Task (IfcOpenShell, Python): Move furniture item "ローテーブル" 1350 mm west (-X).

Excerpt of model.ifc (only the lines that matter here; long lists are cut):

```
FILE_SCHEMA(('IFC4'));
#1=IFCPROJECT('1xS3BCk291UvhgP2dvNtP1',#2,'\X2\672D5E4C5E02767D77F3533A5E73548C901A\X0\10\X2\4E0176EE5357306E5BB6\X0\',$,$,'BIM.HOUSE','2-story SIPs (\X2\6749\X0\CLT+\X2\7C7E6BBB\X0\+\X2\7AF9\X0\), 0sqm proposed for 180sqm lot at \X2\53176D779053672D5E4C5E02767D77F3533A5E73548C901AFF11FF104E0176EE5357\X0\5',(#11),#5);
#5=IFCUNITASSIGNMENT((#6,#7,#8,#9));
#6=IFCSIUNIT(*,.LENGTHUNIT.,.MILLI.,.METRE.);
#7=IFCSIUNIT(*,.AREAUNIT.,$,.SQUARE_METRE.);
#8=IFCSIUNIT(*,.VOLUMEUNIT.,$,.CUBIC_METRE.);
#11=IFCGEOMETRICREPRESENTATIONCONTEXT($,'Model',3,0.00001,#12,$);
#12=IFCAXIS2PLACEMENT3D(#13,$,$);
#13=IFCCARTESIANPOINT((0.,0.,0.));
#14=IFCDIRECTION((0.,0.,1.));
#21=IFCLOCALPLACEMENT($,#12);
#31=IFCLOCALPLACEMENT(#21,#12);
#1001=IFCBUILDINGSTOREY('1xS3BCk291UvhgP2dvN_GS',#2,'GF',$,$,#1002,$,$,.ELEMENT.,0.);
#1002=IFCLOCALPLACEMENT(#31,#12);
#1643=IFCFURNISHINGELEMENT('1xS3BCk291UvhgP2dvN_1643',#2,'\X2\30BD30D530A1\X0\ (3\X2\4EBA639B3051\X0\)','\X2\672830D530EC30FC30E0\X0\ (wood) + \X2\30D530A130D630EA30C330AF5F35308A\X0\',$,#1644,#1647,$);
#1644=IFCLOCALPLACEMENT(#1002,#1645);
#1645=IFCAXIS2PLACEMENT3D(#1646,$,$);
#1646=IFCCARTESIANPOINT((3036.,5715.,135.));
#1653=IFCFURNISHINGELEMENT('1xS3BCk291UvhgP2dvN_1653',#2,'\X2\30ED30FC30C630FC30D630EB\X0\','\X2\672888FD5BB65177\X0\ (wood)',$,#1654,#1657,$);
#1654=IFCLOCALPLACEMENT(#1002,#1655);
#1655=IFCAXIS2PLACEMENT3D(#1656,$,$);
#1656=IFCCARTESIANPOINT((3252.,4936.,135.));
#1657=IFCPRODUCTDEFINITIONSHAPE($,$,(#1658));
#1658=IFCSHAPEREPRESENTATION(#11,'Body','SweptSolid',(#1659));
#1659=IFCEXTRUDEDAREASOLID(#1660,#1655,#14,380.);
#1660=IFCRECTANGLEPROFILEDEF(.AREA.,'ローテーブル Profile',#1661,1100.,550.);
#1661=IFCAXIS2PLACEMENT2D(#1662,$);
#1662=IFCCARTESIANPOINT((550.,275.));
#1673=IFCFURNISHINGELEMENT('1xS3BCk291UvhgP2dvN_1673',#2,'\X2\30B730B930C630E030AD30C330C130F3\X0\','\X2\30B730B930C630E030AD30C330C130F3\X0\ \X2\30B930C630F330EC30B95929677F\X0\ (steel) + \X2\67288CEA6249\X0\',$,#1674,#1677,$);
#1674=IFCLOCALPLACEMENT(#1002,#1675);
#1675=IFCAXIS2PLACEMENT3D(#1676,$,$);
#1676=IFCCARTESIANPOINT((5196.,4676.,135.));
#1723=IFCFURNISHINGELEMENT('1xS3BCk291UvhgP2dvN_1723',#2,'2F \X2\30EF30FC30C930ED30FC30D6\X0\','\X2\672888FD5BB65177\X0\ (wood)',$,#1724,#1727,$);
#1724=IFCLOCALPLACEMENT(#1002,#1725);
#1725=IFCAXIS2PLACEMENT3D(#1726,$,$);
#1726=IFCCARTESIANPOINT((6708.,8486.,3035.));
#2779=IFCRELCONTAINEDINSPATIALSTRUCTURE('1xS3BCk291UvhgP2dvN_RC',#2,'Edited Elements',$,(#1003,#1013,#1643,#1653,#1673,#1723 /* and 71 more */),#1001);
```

```python
import ifcopenshell
import ifcopenshell.api.geometry
import ifcopenshell.util.placement
import ifcopenshell.util.unit

model = ifcopenshell.open("model.ifc")
unit_scale = ifcopenshell.util.unit.calculate_unit_scale(model)

item = model.by_guid("1xS3BCk291UvhgP2dvN_1653")
matrix = ifcopenshell.util.placement.get_local_placement(item.ObjectPlacement)
matrix[0, 3] -= 1.35 / unit_scale
ifcopenshell.api.geometry.edit_object_placement(model, product=item, matrix=matrix, is_si=False)

print(ifcopenshell.util.placement.get_local_placement(item.ObjectPlacement).round(3) + 0.0)

model.write("model_edited.ifc")
```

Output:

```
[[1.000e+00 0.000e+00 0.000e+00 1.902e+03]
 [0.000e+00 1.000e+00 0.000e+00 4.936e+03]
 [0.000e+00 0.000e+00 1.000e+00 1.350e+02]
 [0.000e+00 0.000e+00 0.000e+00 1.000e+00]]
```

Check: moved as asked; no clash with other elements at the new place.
